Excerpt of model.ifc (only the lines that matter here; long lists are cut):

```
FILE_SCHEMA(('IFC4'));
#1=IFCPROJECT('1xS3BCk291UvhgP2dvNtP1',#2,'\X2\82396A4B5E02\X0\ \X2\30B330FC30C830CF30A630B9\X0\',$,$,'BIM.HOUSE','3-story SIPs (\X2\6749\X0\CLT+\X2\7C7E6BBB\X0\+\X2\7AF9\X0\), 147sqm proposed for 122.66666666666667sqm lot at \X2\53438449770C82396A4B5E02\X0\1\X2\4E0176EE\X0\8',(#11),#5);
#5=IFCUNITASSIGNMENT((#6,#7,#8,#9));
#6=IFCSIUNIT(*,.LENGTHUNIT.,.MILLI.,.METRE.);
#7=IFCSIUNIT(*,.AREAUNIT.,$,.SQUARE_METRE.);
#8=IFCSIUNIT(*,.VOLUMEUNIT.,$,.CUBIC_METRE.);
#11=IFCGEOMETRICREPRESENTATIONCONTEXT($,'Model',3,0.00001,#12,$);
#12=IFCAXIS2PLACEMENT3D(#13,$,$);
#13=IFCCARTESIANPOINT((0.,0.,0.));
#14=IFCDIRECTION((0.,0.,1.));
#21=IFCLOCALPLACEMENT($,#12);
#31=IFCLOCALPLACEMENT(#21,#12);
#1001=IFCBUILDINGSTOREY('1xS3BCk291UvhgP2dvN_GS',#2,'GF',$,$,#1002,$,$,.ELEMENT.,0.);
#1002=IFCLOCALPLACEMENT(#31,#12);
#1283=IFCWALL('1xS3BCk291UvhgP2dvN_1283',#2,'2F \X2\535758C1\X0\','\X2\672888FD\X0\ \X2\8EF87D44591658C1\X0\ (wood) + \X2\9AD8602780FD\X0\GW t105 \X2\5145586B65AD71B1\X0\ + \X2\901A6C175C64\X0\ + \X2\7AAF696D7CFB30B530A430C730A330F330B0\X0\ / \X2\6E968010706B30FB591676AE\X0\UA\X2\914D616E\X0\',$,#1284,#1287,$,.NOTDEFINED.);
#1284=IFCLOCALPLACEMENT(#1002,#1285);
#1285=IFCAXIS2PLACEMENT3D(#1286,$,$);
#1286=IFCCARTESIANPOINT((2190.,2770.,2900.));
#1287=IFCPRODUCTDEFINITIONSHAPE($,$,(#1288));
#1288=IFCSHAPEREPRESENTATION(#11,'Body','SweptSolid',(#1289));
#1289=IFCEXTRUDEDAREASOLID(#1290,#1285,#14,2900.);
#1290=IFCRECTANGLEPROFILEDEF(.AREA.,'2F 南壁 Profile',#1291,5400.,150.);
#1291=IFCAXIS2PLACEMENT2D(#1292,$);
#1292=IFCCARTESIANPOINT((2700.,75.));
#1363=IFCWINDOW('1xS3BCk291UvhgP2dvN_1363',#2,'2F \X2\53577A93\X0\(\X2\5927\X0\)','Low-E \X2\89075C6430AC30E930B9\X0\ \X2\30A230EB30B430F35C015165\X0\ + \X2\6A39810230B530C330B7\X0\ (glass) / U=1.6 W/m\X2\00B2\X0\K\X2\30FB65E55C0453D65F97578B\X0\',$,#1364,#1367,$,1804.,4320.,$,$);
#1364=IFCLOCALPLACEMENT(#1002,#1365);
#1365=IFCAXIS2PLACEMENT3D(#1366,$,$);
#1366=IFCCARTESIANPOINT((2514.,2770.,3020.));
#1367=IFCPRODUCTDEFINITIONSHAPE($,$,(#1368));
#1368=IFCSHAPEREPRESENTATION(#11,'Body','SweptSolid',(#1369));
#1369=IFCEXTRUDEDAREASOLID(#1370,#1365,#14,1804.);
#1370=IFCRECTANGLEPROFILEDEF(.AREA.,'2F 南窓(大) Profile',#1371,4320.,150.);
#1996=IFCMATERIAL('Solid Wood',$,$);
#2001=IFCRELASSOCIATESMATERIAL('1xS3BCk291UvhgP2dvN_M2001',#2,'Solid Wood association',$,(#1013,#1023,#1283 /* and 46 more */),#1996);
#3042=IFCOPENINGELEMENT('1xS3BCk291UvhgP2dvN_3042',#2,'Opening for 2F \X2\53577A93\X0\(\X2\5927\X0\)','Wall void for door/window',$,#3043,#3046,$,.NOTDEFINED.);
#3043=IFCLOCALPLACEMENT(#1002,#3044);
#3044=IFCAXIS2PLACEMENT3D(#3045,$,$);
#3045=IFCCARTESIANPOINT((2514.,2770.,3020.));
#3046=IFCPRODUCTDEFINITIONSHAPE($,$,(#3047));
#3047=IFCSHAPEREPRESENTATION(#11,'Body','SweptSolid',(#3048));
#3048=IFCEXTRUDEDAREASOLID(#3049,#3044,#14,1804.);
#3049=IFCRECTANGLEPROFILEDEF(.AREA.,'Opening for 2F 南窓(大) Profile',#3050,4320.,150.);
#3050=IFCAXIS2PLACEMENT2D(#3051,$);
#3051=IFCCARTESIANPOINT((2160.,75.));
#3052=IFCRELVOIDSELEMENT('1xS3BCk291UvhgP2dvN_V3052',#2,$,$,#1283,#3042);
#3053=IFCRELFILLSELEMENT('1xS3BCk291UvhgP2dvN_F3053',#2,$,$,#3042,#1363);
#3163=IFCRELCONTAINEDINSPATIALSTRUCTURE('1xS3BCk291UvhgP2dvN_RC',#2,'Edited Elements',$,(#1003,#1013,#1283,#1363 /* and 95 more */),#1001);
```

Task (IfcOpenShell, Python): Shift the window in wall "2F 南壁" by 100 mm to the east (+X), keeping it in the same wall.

```python
import ifcopenshell
import ifcopenshell.api.geometry
import ifcopenshell.util.placement

model = ifcopenshell.open("model.ifc")

window = model.by_guid("1xS3BCk291UvhgP2dvN_1363")
opening = window.FillsVoids[0].RelatingOpeningElement
wall = opening.VoidsElements[0].RelatingBuildingElement

wall_matrix = ifcopenshell.util.placement.get_local_placement(wall.ObjectPlacement)
shift = wall_matrix[:3, 0] * 100.0
before = ifcopenshell.util.placement.get_local_placement(window.ObjectPlacement)[:3, 3].copy()

# The window is not placed relative to its opening, so move both.
for product in (opening, window):
    matrix = ifcopenshell.util.placement.get_local_placement(product.ObjectPlacement)
    matrix[:3, 3] += shift
    ifcopenshell.api.geometry.edit_object_placement(model, product=product, matrix=matrix, is_si=False)

after = ifcopenshell.util.placement.get_local_placement(window.ObjectPlacement)[:3, 3]
print("window moved by", (after - before).round(3) + 0.0)

model.write("model_edited.ifc")
```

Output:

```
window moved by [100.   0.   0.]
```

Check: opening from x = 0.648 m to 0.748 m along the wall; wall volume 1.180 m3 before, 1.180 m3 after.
